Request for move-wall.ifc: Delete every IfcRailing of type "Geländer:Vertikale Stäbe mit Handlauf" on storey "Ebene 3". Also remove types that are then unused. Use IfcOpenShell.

First a look at what the model holds.

```python
import ifcopenshell
import ifcopenshell.util.element

model = ifcopenshell.open("move-wall.ifc")
print(model.schema)
storey = next(s for s in model.by_type("IfcBuildingStorey") if s.Name == "Ebene 3")
railings = [e for e in ifcopenshell.util.element.get_decomposition(storey) if e.is_a("IfcRailing")]
seen = {}
for e in railings:
    element_type = ifcopenshell.util.element.get_type(e)
    name = element_type.Name if element_type not in (None, e) else None
    seen[name] = seen.get(name, 0) + 1
for name, count in sorted(seen.items(), key=str):
    print(count, "x", name)
```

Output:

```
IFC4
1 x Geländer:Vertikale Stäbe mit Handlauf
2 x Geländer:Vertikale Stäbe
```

```python
import ifcopenshell
import ifcopenshell.api.root
import ifcopenshell.util.element

model = ifcopenshell.open("move-wall.ifc")

storey = next(s for s in model.by_type("IfcBuildingStorey") if s.Name == "Ebene 3")
railings = [e for e in ifcopenshell.util.element.get_decomposition(storey) if e.is_a("IfcRailing")]
targets = [e for e in railings if (t := ifcopenshell.util.element.get_type(e)) not in (None, e) and t.Name == "Geländer:Vertikale Stäbe mit Handlauf"]
types = {ifcopenshell.util.element.get_type(e) for e in targets} - {None, *targets}

for e in targets:
    ifcopenshell.api.root.remove_product(model, product=e)
print(len(targets), "removed")

unused = [t for t in types if not ifcopenshell.util.element.get_types(t)]
for t in unused:
    ifcopenshell.api.root.remove_product(model, product=t)
print(len(unused), "unused types removed")

model.write("move-wall-out.ifc")
```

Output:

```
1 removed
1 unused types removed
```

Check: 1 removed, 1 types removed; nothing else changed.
